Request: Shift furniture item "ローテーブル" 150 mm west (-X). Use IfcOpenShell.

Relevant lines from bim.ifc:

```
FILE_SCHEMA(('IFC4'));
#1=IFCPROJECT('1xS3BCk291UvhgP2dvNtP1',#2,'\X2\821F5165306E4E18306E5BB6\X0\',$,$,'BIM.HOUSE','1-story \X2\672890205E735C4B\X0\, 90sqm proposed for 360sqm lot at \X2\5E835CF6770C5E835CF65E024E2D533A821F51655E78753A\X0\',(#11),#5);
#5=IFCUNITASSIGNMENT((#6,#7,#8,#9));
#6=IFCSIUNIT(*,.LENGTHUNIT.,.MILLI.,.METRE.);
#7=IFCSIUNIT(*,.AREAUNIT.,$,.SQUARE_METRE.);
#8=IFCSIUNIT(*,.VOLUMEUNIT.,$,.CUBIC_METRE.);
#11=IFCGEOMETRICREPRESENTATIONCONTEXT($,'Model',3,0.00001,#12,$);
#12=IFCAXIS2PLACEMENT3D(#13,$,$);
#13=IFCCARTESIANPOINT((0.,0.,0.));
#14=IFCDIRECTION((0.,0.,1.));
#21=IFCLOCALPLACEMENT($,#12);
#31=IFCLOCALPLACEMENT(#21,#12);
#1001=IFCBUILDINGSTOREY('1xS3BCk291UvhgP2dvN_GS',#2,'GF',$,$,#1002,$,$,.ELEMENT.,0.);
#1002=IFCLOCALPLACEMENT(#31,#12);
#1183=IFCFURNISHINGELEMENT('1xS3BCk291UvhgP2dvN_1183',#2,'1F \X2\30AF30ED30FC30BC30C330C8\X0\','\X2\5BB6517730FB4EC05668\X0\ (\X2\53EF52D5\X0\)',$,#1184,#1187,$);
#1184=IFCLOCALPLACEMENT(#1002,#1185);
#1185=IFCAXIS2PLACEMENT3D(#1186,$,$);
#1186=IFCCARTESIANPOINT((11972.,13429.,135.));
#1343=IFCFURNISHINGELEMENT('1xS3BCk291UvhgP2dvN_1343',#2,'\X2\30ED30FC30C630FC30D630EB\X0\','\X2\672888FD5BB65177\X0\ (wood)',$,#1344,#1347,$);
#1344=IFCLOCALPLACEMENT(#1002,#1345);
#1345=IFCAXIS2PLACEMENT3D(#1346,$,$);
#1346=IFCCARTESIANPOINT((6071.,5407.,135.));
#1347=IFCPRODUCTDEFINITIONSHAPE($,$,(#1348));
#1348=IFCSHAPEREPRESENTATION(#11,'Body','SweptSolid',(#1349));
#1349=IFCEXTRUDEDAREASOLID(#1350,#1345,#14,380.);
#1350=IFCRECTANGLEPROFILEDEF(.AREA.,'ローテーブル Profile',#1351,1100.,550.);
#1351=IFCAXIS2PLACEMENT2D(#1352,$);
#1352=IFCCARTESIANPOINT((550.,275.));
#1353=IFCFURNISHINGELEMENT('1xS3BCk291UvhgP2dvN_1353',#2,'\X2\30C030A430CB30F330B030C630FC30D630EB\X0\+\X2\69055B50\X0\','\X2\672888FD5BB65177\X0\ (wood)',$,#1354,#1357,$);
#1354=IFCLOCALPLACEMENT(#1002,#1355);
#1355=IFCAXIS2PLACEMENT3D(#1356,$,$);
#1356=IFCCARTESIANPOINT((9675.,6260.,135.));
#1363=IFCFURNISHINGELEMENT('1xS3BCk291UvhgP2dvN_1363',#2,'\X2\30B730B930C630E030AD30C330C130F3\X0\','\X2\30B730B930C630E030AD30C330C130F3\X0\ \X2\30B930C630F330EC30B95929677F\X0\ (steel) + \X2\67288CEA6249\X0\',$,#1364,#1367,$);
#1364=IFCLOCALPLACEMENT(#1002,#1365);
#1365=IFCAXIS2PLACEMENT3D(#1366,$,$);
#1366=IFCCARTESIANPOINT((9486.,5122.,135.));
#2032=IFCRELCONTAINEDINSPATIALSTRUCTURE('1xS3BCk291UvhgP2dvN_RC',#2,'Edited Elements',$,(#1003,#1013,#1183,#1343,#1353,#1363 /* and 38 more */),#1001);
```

```python
import ifcopenshell
import ifcopenshell.api.geometry
import ifcopenshell.util.placement

model = ifcopenshell.open("bim.ifc")

item = model.by_id(1343)
matrix = ifcopenshell.util.placement.get_local_placement(item.ObjectPlacement)
matrix[0, 3] -= 150.0
ifcopenshell.api.geometry.edit_object_placement(model, product=item, matrix=matrix, is_si=False)

print(ifcopenshell.util.placement.get_local_placement(item.ObjectPlacement).round(3) + 0.0)

model.write("bim_edited.ifc")
```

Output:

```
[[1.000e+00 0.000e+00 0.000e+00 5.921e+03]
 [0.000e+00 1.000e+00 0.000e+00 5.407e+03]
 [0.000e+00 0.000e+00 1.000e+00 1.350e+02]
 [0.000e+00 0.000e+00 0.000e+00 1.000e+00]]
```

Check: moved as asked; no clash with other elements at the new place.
